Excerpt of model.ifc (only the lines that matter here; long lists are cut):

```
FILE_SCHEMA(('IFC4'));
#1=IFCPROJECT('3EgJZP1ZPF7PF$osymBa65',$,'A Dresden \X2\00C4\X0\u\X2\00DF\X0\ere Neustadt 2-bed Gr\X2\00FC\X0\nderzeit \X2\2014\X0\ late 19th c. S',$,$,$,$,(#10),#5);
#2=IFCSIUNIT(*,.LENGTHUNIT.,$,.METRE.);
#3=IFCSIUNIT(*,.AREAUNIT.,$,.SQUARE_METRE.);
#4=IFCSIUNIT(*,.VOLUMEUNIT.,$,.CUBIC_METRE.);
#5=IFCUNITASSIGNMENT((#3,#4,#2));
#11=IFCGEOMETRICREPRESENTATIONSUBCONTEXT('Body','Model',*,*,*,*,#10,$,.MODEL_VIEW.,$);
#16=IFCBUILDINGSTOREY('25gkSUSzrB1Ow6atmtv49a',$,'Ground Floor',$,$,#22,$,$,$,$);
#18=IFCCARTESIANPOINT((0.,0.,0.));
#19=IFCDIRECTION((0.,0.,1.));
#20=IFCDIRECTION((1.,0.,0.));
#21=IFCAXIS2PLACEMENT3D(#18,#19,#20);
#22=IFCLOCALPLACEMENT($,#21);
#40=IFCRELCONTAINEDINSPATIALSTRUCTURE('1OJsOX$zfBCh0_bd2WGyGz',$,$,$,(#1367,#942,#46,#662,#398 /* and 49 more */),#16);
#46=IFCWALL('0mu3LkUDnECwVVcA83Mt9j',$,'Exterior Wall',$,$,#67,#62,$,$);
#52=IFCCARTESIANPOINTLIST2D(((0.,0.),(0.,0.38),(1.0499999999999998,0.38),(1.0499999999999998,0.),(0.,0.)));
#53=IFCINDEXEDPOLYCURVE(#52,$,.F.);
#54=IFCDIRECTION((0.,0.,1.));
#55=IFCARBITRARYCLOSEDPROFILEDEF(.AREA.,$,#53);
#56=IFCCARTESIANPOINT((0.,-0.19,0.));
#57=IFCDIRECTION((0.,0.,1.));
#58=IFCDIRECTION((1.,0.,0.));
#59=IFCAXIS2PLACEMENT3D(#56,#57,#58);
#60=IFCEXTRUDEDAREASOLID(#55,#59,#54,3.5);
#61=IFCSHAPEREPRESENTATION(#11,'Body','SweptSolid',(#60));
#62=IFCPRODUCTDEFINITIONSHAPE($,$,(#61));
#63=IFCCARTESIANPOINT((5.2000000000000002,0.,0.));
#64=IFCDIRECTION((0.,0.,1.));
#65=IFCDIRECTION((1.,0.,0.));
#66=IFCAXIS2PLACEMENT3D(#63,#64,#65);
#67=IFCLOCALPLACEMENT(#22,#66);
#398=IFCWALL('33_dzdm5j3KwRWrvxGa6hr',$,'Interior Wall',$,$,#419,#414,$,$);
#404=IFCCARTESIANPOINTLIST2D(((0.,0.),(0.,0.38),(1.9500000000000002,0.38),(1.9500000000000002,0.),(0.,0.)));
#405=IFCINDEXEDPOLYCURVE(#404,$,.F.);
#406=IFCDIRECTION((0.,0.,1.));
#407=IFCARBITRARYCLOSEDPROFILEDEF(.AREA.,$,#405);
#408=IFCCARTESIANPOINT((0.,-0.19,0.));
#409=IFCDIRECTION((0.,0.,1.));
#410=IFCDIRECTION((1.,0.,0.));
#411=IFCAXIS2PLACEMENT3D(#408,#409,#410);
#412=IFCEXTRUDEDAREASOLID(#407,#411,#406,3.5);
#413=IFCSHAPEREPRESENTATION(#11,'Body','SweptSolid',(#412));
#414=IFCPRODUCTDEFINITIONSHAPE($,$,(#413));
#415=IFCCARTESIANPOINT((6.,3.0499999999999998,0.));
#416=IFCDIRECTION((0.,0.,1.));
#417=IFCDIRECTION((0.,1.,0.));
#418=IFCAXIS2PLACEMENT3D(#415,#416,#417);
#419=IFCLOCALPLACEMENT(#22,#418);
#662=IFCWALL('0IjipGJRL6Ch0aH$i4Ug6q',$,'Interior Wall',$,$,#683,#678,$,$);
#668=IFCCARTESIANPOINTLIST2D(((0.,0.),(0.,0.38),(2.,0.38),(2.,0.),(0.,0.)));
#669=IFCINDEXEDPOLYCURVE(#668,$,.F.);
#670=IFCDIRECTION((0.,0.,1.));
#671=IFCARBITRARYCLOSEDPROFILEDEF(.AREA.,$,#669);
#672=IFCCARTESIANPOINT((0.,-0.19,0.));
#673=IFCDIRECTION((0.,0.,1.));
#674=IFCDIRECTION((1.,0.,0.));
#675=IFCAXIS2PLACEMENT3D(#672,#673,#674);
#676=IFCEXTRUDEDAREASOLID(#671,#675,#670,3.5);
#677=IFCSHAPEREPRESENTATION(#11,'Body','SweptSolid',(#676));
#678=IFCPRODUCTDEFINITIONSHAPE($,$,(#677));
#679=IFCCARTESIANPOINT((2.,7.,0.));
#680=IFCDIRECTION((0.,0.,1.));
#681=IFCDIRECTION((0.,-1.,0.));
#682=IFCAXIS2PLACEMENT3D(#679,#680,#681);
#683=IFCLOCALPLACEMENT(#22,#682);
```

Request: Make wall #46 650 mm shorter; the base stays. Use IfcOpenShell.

```python
import ifcopenshell
import ifcopenshell.geom
import ifcopenshell.util.representation
import ifcopenshell.util.shape
import ifcopenshell.util.unit

model = ifcopenshell.open("model.ifc")
unit_scale = ifcopenshell.util.unit.calculate_unit_scale(model)
settings = ifcopenshell.geom.settings()


def volume(element):
    """Net volume in cubic metres, openings subtracted."""
    shape = ifcopenshell.geom.create_shape(settings, element)
    return ifcopenshell.util.shape.get_volume(shape.geometry)


wall = model.by_guid("0mu3LkUDnECwVVcA83Mt9j")
before = volume(wall)

body = ifcopenshell.util.representation.get_representation(wall, "Model", "Body")
solid = body.Items[0]
old_height = solid.Depth
solid.Depth -= 0.65 / unit_scale
after = volume(wall)

print(f"height {old_height:g} -> {solid.Depth:g}, volume {before:.3f} -> {after:.3f} m3")

model.write("model-out.ifc")
```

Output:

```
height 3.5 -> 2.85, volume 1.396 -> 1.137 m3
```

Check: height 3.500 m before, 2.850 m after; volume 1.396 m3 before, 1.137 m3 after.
